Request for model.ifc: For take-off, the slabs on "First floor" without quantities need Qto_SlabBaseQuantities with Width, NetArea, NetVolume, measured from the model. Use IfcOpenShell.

First a look at what the model holds.

```python
import ifcopenshell
import ifcopenshell.util.element
import ifcopenshell.util.unit

model = ifcopenshell.open("model.ifc")
print(model.schema)
for unit_type in ("LENGTHUNIT", "AREAUNIT", "VOLUMEUNIT"):
    print(unit_type, ifcopenshell.util.unit.calculate_unit_scale(model, unit_type))
storey = next(s for s in model.by_type("IfcBuildingStorey") if s.Name == "First floor")
slabs = [e for e in ifcopenshell.util.element.get_decomposition(storey) if e.is_a("IfcSlab")]
for e in sorted(slabs, key=lambda e: e.id()):
    print(e.id(), e.is_a(), e.Name, list(ifcopenshell.util.element.get_psets(e, qtos_only=True)), sep=" | ")
```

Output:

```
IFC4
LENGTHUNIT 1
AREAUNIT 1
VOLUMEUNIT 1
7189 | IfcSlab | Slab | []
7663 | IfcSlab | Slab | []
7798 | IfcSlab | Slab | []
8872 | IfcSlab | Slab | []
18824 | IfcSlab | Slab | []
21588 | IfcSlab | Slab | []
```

```python
import ifcopenshell
import ifcopenshell.api.pset
import ifcopenshell.geom
import ifcopenshell.util.element
import ifcopenshell.util.shape
import ifcopenshell.util.unit

model = ifcopenshell.open("model.ifc")
unit_scale = ifcopenshell.util.unit.calculate_unit_scale(model)
area_scale = ifcopenshell.util.unit.calculate_unit_scale(model, "AREAUNIT")
volume_scale = ifcopenshell.util.unit.calculate_unit_scale(model, "VOLUMEUNIT")
settings = ifcopenshell.geom.settings()

storey = next(s for s in model.by_type("IfcBuildingStorey") if s.Name == "First floor")
slabs = [e for e in ifcopenshell.util.element.get_decomposition(storey) if e.is_a("IfcSlab")]

for e in sorted(slabs, key=lambda e: e.id()):
    if ifcopenshell.util.element.get_psets(e, qtos_only=True, should_inherit=False):
        continue
    # Geometry comes back in metres, in the element's own axes.
    shape = ifcopenshell.geom.create_shape(settings, e)
    values = {
        "Width": ifcopenshell.util.shape.get_z(shape.geometry) / unit_scale,
        "NetArea": ifcopenshell.util.shape.get_footprint_area(shape.geometry) / area_scale,
        "NetVolume": ifcopenshell.util.shape.get_volume(shape.geometry) / volume_scale,
    }
    qto = ifcopenshell.api.pset.add_qto(model, product=e, name="Qto_SlabBaseQuantities")
    ifcopenshell.api.pset.edit_qto(model, qto=qto, properties=values)
    print(e.id(), {k: round(v, 3) for k, v in values.items()})

model.write("model_edited.ifc")
```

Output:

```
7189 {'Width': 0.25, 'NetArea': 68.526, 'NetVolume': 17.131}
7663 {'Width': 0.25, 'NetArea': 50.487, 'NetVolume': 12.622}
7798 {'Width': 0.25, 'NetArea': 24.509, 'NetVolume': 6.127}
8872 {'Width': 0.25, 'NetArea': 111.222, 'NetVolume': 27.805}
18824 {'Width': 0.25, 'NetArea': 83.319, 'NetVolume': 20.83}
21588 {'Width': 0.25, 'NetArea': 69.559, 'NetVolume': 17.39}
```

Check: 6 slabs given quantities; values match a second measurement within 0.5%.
